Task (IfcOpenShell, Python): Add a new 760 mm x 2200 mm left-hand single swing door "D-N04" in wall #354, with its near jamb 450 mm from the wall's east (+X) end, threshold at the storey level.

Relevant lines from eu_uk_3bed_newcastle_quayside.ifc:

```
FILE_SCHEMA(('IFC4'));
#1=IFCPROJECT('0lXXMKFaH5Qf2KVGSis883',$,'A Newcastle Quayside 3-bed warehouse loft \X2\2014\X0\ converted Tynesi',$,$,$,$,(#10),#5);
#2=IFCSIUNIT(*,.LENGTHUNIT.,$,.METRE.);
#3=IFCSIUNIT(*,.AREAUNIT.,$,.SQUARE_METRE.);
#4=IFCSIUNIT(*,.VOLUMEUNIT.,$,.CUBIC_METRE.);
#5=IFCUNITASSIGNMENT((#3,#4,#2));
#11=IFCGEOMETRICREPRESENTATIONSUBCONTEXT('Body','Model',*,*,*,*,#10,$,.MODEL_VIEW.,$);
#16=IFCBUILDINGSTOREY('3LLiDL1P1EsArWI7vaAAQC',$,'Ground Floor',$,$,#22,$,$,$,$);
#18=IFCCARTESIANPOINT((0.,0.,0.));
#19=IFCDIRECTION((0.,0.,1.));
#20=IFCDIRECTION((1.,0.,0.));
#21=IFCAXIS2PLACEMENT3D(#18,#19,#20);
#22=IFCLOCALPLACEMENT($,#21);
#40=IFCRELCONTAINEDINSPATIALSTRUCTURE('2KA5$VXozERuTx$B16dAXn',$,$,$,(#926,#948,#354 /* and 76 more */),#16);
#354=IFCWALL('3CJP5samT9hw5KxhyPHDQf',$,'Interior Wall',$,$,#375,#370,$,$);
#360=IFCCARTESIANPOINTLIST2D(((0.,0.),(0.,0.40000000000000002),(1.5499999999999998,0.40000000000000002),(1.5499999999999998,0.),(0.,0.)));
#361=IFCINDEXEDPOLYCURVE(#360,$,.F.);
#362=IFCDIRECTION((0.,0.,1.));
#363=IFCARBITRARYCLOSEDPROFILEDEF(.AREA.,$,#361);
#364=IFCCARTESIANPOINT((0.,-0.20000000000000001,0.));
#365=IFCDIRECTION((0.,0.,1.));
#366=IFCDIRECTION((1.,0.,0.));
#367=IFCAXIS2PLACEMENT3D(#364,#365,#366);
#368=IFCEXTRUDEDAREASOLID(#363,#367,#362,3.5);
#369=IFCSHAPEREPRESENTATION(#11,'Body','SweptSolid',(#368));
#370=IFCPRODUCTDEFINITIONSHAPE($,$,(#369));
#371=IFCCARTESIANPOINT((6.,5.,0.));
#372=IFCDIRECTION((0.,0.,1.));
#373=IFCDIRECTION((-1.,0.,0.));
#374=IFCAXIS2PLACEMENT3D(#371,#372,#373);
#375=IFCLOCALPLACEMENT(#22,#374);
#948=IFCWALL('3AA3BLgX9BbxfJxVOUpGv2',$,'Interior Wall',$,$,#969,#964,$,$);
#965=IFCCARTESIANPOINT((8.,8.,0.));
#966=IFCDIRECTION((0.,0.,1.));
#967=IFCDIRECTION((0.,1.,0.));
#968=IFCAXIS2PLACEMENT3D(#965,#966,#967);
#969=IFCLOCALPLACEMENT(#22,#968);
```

```python
import numpy as np
import ifcopenshell
import ifcopenshell.api.feature
import ifcopenshell.api.geometry
import ifcopenshell.api.root
import ifcopenshell.api.spatial
import ifcopenshell.geom
import ifcopenshell.util.element
import ifcopenshell.util.placement
import ifcopenshell.util.representation
import ifcopenshell.util.shape
import ifcopenshell.util.unit

model = ifcopenshell.open("eu_uk_3bed_newcastle_quayside.ifc")
unit_scale = ifcopenshell.util.unit.calculate_unit_scale(model)
settings = ifcopenshell.geom.settings()


def volume(element):
    """Net volume in cubic metres, openings subtracted."""
    shape = ifcopenshell.geom.create_shape(settings, element)
    return ifcopenshell.util.shape.get_volume(shape.geometry)


wall = model.by_guid("3CJP5samT9hw5KxhyPHDQf")
storey = ifcopenshell.util.element.get_container(wall, ifc_class="IfcBuildingStorey")
context = ifcopenshell.util.representation.get_context(model, "Model", "Body", "MODEL_VIEW")
before = volume(wall)

width, height, from_end, sill = 0.76, 2.2, 0.45, 0.0  # metres

# The wall runs along its own X axis, and the end named is its -X end.
wall_shape = ifcopenshell.geom.create_shape(settings, wall)
x, y, z = ifcopenshell.util.shape.get_vertices(wall_shape.geometry).T
start = x.min() + from_end
face, thickness = float(y.min()), float(y.max() - y.min())
wall_matrix = ifcopenshell.util.placement.get_local_placement(wall.ObjectPlacement)
level = ifcopenshell.util.placement.get_local_placement(storey.ObjectPlacement)[2, 3]


def in_wall(x, y):
    """Placement at x, y metres in the wall's axes, at sill height."""
    matrix = wall_matrix.copy()
    matrix[:, 3] = wall_matrix @ np.array([x / unit_scale, y / unit_scale, 0.0, 1.0])
    matrix[2, 3] = level + sill / unit_scale
    return matrix


# Opening: a box that overshoots both wall faces by 50 mm.
opening = ifcopenshell.api.root.create_entity(model, ifc_class="IfcOpeningElement", predefined_type="OPENING")
box = ifcopenshell.api.geometry.add_wall_representation(
    model, context=context, length=width, height=height, thickness=thickness + 0.1
)
ifcopenshell.api.geometry.assign_representation(model, product=opening, representation=box)
ifcopenshell.api.geometry.edit_object_placement(model, product=opening, matrix=in_wall(start, face - 0.05), is_si=False)
ifcopenshell.api.feature.add_feature(model, feature=opening, element=wall)

door = ifcopenshell.api.root.create_entity(model, ifc_class="IfcDoor", name="D-N04", predefined_type="DOOR")
door.OverallWidth, door.OverallHeight = width / unit_scale, height / unit_scale
door.OperationType = "SINGLE_SWING_LEFT"
body = ifcopenshell.api.geometry.add_door_representation(
    model,
    context=context,
    overall_width=door.OverallWidth,
    overall_height=door.OverallHeight,
    operation_type="SINGLE_SWING_LEFT",
    lining_properties={"LiningDepth": thickness / unit_scale, "ThresholdDepth": thickness / unit_scale},
)
ifcopenshell.api.geometry.assign_representation(model, product=door, representation=body)
ifcopenshell.api.spatial.assign_container(model, products=[door], relating_structure=storey)
ifcopenshell.api.feature.add_filling(model, opening=opening, element=door)

# The lining spans the wall, so the door starts at the wall face.
ifcopenshell.api.geometry.edit_object_placement(model, product=door, matrix=in_wall(start, face), is_si=False)

after = volume(wall)

print(f"wall volume {before:.3f} -> {after:.3f} m3")

model.write("eu_uk_3bed_newcastle_quayside_edited.ifc")
```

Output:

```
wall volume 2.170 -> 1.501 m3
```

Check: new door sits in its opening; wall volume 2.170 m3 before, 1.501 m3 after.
